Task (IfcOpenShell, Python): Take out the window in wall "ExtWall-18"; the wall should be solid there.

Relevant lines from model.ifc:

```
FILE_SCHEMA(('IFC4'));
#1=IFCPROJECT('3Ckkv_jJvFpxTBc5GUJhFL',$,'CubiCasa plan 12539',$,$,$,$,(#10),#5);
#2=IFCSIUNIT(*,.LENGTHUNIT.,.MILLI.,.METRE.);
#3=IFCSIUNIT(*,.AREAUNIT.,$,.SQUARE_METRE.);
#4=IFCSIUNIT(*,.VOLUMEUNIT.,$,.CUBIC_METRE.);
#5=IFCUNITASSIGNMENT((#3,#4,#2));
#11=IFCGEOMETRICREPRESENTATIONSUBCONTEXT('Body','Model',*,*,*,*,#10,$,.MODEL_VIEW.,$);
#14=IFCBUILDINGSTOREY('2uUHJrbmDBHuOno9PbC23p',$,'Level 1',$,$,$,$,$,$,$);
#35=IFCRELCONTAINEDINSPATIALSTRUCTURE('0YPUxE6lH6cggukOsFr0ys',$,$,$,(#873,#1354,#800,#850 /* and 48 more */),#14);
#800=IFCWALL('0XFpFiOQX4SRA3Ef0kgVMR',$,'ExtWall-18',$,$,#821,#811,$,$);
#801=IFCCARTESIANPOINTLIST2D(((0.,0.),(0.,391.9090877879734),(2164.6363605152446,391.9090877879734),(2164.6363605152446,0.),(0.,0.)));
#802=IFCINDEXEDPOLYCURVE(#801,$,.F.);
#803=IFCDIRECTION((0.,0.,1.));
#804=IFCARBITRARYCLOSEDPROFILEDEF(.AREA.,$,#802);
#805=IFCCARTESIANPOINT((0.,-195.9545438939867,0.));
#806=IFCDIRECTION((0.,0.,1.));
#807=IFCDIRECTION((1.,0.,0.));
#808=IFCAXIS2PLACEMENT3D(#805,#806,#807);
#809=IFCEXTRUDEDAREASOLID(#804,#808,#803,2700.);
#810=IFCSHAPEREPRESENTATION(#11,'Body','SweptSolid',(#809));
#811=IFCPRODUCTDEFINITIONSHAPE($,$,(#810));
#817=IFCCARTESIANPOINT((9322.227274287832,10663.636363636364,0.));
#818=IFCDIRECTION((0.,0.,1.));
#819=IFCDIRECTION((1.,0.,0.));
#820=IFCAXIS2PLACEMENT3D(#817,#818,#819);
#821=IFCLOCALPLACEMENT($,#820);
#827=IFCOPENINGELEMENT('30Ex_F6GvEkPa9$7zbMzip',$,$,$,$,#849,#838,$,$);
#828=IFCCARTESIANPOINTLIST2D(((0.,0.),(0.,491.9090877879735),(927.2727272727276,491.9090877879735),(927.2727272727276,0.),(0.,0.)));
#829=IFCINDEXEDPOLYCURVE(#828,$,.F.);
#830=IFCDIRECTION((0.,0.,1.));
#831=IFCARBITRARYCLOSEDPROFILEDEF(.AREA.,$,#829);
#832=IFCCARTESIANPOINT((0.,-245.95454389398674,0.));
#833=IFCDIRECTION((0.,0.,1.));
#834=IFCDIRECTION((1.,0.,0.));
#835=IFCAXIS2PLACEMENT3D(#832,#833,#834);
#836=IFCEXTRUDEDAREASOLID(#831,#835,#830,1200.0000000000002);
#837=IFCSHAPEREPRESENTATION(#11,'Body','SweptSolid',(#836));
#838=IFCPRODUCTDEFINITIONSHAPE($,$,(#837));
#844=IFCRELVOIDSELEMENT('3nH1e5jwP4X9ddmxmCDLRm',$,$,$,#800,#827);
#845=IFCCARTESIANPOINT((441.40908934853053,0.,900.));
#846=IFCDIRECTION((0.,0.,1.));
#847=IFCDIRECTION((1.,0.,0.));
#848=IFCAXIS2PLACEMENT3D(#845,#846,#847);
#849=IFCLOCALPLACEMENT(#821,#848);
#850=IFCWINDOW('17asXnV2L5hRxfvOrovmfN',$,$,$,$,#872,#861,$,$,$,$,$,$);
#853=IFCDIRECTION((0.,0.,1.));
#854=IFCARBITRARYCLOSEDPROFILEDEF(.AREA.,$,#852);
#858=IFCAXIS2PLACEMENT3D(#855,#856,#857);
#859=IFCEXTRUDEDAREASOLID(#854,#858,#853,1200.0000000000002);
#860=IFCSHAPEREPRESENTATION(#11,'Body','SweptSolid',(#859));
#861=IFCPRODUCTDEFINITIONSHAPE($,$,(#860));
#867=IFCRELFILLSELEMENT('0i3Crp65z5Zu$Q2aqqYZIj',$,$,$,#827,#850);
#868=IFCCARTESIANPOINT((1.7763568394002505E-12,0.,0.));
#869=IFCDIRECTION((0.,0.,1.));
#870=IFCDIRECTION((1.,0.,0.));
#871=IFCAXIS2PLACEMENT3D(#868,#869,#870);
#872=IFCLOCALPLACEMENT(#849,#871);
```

```python
import ifcopenshell
import ifcopenshell.api.feature
import ifcopenshell.api.root
import ifcopenshell.geom
import ifcopenshell.util.shape

model = ifcopenshell.open("model.ifc")
settings = ifcopenshell.geom.settings()


def volume(element):
    """Net volume in cubic metres, openings subtracted."""
    shape = ifcopenshell.geom.create_shape(settings, element)
    return ifcopenshell.util.shape.get_volume(shape.geometry)


window = model.by_id(850)
opening = window.FillsVoids[0].RelatingOpeningElement
wall = opening.VoidsElements[0].RelatingBuildingElement
before = volume(wall)

ifcopenshell.api.root.remove_product(model, product=window)
ifcopenshell.api.feature.remove_feature(model, feature=opening)

after = volume(wall)

print(f"wall volume {before:.3f} -> {after:.3f} m3")

model.write("model_rev.ifc")
```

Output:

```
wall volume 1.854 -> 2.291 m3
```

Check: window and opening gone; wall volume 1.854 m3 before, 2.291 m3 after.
